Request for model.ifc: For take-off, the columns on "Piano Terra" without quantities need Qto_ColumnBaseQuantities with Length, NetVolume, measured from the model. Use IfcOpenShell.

First a look at what the model holds.

```python
import ifcopenshell
import ifcopenshell.util.element
import ifcopenshell.util.unit

model = ifcopenshell.open("model.ifc")
print(model.schema)
for unit_type in ("LENGTHUNIT", "AREAUNIT", "VOLUMEUNIT"):
    print(unit_type, ifcopenshell.util.unit.calculate_unit_scale(model, unit_type))
storey = next(s for s in model.by_type("IfcBuildingStorey") if s.Name == "Piano Terra")
columns = [e for e in ifcopenshell.util.element.get_decomposition(storey) if e.is_a("IfcColumn")]
for e in sorted(columns, key=lambda e: e.id()):
    print(e.id(), e.is_a(), e.Name, list(ifcopenshell.util.element.get_psets(e, qtos_only=True)), sep=" | ")
```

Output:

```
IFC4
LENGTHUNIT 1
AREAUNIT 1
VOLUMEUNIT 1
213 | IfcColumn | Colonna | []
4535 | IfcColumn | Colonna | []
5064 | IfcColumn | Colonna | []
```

```python
import ifcopenshell
import ifcopenshell.api.pset
import ifcopenshell.geom
import ifcopenshell.util.element
import ifcopenshell.util.shape
import ifcopenshell.util.unit

model = ifcopenshell.open("model.ifc")
unit_scale = ifcopenshell.util.unit.calculate_unit_scale(model)
volume_scale = ifcopenshell.util.unit.calculate_unit_scale(model, "VOLUMEUNIT")
settings = ifcopenshell.geom.settings()

storey = next(s for s in model.by_type("IfcBuildingStorey") if s.Name == "Piano Terra")
columns = [e for e in ifcopenshell.util.element.get_decomposition(storey) if e.is_a("IfcColumn")]

for e in sorted(columns, key=lambda e: e.id()):
    if ifcopenshell.util.element.get_psets(e, qtos_only=True, should_inherit=False):
        continue
    # Geometry comes back in metres, in the element's own axes.
    shape = ifcopenshell.geom.create_shape(settings, e)
    values = {
        "Length": ifcopenshell.util.shape.get_z(shape.geometry) / unit_scale,
        "NetVolume": ifcopenshell.util.shape.get_volume(shape.geometry) / volume_scale,
    }
    qto = ifcopenshell.api.pset.add_qto(model, product=e, name="Qto_ColumnBaseQuantities")
    ifcopenshell.api.pset.edit_qto(model, qto=qto, properties=values)
    print(e.id(), {k: round(v, 3) for k, v in values.items()})

model.write("model_v2.ifc")
```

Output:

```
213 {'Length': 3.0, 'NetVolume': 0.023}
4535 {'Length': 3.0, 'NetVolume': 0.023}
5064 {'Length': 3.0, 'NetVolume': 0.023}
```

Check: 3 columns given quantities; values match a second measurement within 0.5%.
